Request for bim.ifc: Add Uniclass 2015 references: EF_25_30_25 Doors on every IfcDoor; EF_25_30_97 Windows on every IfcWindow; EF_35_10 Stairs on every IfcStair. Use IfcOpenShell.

First a look at what the model holds.

```python
import ifcopenshell

model = ifcopenshell.open("bim.ifc")
print(model.schema)
print("classifications:", [c.Name for c in model.by_type("IfcClassification")])
for ifc_class in ("IfcDoor", "IfcRoof", "IfcStair", "IfcWall", "IfcWindow"):
    print(ifc_class, len(model.by_type(ifc_class)))
```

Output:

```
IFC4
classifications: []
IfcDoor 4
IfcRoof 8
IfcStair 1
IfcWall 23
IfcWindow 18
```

```python
import ifcopenshell
import ifcopenshell.api.classification

model = ifcopenshell.open("bim.ifc")

system = ifcopenshell.api.classification.add_classification(model, classification="Uniclass 2015")

codes = {
    "IfcDoor": ("EF_25_30_25", "Doors"),
    "IfcWindow": ("EF_25_30_97", "Windows"),
    "IfcStair": ("EF_35_10", "Stairs"),
}
for ifc_class, (code, name) in codes.items():
    products = model.by_type(ifc_class)
    ifcopenshell.api.classification.add_reference(
        model, products=products, classification=system, identification=code, name=name
    )
    print(code, len(products))

model.write("bim_updated.ifc")
```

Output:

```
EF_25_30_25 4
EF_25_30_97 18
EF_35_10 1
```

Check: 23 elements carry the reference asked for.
